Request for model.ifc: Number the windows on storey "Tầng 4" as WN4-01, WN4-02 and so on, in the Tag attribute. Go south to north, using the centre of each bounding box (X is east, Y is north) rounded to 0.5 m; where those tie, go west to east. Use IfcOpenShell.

First a look at what the model holds.

```python
import ifcopenshell
import ifcopenshell.util.element
import ifcopenshell.util.placement

model = ifcopenshell.open("model.ifc")
print(model.schema)
storey = next(s for s in model.by_type("IfcBuildingStorey") if s.Name == "Tầng 4")
windows = [e for e in ifcopenshell.util.element.get_decomposition(storey) if e.is_a("IfcWindow")]
for e in sorted(windows, key=lambda e: e.id()):
    origin = ifcopenshell.util.placement.get_local_placement(e.ObjectPlacement)[:3, 3]
    print(e.id(), e.Tag, e.Name, origin.round(2) + 0.0, sep=" | ")
```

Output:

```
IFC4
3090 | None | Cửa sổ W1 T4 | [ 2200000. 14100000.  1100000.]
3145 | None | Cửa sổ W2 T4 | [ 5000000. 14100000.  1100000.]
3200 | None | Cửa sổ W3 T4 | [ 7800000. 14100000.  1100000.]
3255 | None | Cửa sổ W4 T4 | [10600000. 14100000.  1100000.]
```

```python
import ifcopenshell
import ifcopenshell.geom
import ifcopenshell.util.element
import ifcopenshell.util.shape

model = ifcopenshell.open("model.ifc")
settings = ifcopenshell.geom.settings()
settings.set("use-world-coords", True)


def centre(element):
    shape = ifcopenshell.geom.create_shape(settings, element)
    return ifcopenshell.util.shape.get_bbox_centroid(shape.geometry)


storey = next(s for s in model.by_type("IfcBuildingStorey") if s.Name == "Tầng 4")
windows = [e for e in ifcopenshell.util.element.get_decomposition(storey) if e.is_a("IfcWindow")]

# Insertion points can sit at a corner or the storey origin, so sort by the geometry (in metres).
centres = {e: centre(e) for e in windows}
windows.sort(key=lambda e: (round(centres[e][1] / 0.5), centres[e][0]))

for i, e in enumerate(windows, start=1):
    number = f"WN4-{i:02d}"
    e.Tag = number
    print(e.id(), number)

model.write("model_rev.ifc")
```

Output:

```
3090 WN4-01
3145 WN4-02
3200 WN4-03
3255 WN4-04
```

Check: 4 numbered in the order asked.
